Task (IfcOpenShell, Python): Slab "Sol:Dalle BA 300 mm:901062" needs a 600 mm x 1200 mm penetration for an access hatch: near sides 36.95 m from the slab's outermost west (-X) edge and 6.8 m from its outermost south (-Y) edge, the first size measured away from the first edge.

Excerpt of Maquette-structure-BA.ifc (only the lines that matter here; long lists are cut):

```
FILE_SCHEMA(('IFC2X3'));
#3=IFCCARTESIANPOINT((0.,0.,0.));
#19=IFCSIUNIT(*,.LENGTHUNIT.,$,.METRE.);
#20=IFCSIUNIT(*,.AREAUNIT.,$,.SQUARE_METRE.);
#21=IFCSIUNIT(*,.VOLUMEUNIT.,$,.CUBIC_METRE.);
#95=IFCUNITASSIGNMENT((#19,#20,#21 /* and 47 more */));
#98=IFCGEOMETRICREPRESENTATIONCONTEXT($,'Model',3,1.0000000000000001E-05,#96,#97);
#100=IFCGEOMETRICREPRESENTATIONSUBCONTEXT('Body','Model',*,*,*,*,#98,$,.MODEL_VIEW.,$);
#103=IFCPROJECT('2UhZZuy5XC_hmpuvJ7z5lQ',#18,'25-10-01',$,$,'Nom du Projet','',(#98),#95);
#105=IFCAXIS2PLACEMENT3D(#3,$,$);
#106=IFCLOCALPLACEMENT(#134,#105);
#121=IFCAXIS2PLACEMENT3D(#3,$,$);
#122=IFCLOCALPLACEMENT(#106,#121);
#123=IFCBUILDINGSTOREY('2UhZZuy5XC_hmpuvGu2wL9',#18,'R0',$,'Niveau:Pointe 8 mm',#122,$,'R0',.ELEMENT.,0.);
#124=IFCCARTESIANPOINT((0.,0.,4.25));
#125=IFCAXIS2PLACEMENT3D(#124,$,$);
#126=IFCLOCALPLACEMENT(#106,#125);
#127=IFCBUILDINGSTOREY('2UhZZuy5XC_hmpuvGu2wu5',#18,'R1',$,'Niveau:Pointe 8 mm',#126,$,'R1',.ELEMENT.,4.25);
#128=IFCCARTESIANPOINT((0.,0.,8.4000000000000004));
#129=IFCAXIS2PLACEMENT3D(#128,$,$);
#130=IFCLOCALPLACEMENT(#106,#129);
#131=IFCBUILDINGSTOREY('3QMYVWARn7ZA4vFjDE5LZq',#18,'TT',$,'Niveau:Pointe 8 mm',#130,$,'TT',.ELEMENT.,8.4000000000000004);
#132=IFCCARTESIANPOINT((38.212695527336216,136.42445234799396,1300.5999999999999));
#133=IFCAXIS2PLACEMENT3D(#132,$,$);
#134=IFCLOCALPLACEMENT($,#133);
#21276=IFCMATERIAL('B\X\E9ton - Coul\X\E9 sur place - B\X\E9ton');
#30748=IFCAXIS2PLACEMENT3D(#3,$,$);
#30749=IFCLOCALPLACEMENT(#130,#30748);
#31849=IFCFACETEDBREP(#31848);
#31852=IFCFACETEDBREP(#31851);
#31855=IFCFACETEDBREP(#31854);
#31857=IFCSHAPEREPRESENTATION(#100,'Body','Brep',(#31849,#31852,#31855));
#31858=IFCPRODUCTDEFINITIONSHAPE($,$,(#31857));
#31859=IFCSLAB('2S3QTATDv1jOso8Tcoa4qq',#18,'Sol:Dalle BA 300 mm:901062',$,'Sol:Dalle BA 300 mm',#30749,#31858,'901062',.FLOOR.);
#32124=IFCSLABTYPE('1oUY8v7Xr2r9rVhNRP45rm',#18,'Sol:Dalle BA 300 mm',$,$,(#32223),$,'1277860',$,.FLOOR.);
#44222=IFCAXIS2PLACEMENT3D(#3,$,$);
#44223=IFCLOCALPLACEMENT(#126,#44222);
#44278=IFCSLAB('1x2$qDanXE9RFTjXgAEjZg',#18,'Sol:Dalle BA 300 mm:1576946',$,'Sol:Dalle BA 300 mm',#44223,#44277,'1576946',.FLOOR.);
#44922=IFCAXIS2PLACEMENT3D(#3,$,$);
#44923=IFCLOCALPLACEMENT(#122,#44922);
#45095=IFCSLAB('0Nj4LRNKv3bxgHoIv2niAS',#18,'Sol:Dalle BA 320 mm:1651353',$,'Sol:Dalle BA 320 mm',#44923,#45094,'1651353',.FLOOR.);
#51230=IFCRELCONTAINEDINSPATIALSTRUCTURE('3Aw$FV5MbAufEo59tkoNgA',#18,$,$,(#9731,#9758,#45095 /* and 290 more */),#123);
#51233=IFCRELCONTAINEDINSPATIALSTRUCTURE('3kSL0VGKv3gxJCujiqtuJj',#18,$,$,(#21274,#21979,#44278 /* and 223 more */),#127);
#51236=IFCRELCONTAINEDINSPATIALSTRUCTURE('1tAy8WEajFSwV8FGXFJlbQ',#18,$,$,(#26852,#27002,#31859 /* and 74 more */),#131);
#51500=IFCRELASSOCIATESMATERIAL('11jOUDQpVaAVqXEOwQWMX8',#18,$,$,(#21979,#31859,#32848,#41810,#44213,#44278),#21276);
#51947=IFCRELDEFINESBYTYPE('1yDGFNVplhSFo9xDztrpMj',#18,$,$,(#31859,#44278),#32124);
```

```python
import numpy as np
import ifcopenshell
import ifcopenshell.api.feature
import ifcopenshell.api.geometry
import ifcopenshell.api.root
import ifcopenshell.geom
import ifcopenshell.util.placement
import ifcopenshell.util.representation
import ifcopenshell.util.shape
import ifcopenshell.util.unit

model = ifcopenshell.open("Maquette-structure-BA.ifc")
unit_scale = ifcopenshell.util.unit.calculate_unit_scale(model)
settings = ifcopenshell.geom.settings()


def volume(element):
    """Net volume in cubic metres, openings subtracted."""
    shape = ifcopenshell.geom.create_shape(settings, element)
    return ifcopenshell.util.shape.get_volume(shape.geometry)


slab = model.by_guid("2S3QTATDv1jOso8Tcoa4qq")
before = volume(slab)

# Extent in the slab's own axes, in metres. The edges named are its -X and -Y sides.
slab_shape = ifcopenshell.geom.create_shape(settings, slab)
vertices = ifcopenshell.util.shape.get_vertices(slab_shape.geometry)
x_min, y_min, bottom = vertices.min(axis=0)
top = vertices[:, 2].max()

opening = ifcopenshell.api.root.create_entity(model, ifc_class="IfcOpeningElement", name="Access hatch opening")
context = ifcopenshell.util.representation.get_context(model, "Model", "Body", "MODEL_VIEW")
width, depth = 0.6, 1.2
outline = [(0.0, 0.0), (width, 0.0), (width, depth), (0.0, depth), (0.0, 0.0)]
# Overshoot both faces by 50 mm so the cut is clean.
shape = ifcopenshell.api.geometry.add_slab_representation(
    model, context=context, depth=top - bottom + 0.1, polyline=outline
)
ifcopenshell.api.geometry.assign_representation(model, product=opening, representation=shape)

matrix = ifcopenshell.util.placement.get_local_placement(slab.ObjectPlacement)
matrix[:, 3] = matrix @ np.append(np.array([x_min + 36.95, y_min + 6.8, bottom - 0.05]) / unit_scale, 1.0)
ifcopenshell.api.geometry.edit_object_placement(model, product=opening, matrix=matrix, is_si=False)
ifcopenshell.api.feature.add_feature(model, feature=opening, element=slab)

after = volume(slab)

print(f"slab volume {before:.3f} -> {after:.3f} m3")

model.write("Maquette-structure-BA_rev.ifc")
```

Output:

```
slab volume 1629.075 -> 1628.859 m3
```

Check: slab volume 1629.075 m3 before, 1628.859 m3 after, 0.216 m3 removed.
